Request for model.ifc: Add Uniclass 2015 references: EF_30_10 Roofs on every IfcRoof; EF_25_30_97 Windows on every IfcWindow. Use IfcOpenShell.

First a look at what the model holds.

```python
import ifcopenshell

model = ifcopenshell.open("model.ifc")
print(model.schema)
print("classifications:", [c.Name for c in model.by_type("IfcClassification")])
for ifc_class in ("IfcDoor", "IfcRoof", "IfcStair", "IfcWall", "IfcWindow"):
    print(ifc_class, len(model.by_type(ifc_class)))
```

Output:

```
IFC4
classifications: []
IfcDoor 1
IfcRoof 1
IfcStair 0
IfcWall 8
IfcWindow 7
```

```python
import ifcopenshell
import ifcopenshell.api.classification

model = ifcopenshell.open("model.ifc")

system = ifcopenshell.api.classification.add_classification(model, classification="Uniclass 2015")

codes = {
    "IfcRoof": ("EF_30_10", "Roofs"),
    "IfcWindow": ("EF_25_30_97", "Windows"),
}
for ifc_class, (code, name) in codes.items():
    products = model.by_type(ifc_class)
    ifcopenshell.api.classification.add_reference(
        model, products=products, classification=system, identification=code, name=name
    )
    print(code, len(products))

model.write("model_edited.ifc")
```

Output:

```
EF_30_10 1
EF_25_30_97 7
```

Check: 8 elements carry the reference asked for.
